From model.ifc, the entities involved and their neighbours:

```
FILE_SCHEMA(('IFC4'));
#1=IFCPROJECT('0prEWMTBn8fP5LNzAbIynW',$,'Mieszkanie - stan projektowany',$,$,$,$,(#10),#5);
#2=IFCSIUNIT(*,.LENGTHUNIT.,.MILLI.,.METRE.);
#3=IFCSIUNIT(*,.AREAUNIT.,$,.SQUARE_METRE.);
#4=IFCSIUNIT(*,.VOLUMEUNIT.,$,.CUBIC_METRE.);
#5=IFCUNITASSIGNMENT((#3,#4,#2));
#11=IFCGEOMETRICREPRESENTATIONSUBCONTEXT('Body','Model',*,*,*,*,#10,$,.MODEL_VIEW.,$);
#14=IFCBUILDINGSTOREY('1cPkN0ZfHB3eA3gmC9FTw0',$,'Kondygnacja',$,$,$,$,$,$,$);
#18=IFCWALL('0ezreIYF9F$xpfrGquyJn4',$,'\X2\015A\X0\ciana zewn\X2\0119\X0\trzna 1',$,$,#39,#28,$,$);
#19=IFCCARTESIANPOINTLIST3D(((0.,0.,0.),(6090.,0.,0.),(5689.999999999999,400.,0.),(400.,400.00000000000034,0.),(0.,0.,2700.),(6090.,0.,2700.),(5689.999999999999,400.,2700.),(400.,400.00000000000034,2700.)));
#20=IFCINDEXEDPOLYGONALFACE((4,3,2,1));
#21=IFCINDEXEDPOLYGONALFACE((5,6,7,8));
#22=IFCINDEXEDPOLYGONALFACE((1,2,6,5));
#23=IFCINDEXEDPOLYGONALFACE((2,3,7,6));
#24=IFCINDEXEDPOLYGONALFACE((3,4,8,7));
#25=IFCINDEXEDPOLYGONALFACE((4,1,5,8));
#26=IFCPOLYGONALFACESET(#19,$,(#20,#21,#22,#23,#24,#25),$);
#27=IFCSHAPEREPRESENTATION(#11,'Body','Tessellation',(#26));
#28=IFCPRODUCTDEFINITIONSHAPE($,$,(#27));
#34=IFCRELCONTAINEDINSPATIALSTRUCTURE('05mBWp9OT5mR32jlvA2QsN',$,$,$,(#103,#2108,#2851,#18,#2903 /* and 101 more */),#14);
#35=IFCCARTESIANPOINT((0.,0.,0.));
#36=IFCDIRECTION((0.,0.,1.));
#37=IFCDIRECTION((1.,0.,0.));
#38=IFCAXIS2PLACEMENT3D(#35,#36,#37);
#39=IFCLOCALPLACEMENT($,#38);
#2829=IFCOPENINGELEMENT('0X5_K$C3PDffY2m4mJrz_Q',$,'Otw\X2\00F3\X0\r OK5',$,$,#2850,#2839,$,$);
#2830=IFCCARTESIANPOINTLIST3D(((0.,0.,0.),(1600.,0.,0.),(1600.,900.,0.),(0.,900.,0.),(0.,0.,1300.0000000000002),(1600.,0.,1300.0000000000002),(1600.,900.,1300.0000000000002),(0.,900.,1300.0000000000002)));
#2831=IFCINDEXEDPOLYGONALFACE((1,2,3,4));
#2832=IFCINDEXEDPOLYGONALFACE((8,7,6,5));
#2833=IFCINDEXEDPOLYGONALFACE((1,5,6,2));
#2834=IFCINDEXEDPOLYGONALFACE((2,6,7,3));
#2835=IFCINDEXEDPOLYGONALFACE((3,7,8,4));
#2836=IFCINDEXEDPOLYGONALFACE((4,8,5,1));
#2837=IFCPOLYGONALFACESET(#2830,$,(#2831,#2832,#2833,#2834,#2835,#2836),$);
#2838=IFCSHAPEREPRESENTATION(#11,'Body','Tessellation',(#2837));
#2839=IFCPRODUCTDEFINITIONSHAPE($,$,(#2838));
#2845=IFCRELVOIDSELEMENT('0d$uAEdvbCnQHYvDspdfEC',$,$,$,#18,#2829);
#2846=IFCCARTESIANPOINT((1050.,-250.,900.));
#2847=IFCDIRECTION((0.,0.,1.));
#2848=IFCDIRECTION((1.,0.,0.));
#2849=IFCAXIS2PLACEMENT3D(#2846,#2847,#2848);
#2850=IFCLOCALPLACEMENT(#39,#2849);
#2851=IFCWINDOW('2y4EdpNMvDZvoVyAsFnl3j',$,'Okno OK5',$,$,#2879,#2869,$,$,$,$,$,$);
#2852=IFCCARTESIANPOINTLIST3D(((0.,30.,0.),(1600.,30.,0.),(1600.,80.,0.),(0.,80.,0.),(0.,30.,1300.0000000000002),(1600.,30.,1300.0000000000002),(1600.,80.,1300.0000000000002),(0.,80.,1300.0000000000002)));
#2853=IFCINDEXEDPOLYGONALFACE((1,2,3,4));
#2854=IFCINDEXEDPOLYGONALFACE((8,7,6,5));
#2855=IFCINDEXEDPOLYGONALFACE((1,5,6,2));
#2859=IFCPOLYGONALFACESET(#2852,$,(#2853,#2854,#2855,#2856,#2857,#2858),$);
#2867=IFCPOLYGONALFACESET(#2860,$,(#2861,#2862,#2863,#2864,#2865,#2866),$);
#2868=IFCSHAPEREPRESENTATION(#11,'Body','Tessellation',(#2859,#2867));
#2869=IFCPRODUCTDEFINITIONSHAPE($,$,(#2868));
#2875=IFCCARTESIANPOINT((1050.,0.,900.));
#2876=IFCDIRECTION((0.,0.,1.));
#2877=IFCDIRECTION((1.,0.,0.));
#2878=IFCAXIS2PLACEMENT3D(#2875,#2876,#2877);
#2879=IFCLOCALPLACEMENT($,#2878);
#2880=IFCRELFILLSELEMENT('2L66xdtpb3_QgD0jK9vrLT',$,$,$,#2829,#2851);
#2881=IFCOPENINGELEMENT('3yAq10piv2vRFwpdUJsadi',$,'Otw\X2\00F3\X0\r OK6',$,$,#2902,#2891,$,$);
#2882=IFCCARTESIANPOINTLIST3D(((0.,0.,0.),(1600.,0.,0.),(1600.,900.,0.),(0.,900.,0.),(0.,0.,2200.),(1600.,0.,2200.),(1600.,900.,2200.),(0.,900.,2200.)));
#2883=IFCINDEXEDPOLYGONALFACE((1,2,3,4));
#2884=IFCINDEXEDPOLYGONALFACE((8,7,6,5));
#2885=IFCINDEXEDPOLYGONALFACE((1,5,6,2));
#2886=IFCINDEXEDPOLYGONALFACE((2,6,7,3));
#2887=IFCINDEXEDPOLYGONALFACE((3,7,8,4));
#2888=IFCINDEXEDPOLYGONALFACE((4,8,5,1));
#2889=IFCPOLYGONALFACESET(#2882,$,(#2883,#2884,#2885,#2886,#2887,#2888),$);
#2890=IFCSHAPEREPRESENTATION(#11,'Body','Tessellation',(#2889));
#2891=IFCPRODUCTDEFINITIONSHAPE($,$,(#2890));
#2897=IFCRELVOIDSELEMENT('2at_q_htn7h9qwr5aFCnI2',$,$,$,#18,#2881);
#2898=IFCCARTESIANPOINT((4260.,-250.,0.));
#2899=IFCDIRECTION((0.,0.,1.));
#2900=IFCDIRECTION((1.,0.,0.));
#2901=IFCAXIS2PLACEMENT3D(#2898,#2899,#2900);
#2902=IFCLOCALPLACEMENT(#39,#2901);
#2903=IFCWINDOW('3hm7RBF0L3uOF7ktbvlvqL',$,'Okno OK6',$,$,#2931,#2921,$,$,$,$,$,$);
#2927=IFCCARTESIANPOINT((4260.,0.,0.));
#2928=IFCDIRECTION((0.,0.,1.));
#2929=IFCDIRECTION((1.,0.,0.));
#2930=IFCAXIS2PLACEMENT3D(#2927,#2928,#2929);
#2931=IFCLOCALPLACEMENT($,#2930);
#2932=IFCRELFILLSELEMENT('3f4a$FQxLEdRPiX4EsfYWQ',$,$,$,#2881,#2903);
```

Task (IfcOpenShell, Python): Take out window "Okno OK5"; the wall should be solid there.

```python
import ifcopenshell
import ifcopenshell.api.feature
import ifcopenshell.api.root
import ifcopenshell.geom
import ifcopenshell.util.shape

model = ifcopenshell.open("model.ifc")
settings = ifcopenshell.geom.settings()


def volume(element):
    """Net volume in cubic metres, openings subtracted."""
    shape = ifcopenshell.geom.create_shape(settings, element)
    return ifcopenshell.util.shape.get_volume(shape.geometry)


window = model.by_guid("2y4EdpNMvDZvoVyAsFnl3j")
opening = window.FillsVoids[0].RelatingOpeningElement
wall = opening.VoidsElements[0].RelatingBuildingElement
before = volume(wall)

ifcopenshell.api.root.remove_product(model, product=window)
ifcopenshell.api.feature.remove_feature(model, feature=opening)

after = volume(wall)

print(f"wall volume {before:.3f} -> {after:.3f} m3")

model.write("model_v2.ifc")
```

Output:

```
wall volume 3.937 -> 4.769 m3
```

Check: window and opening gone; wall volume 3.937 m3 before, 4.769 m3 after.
